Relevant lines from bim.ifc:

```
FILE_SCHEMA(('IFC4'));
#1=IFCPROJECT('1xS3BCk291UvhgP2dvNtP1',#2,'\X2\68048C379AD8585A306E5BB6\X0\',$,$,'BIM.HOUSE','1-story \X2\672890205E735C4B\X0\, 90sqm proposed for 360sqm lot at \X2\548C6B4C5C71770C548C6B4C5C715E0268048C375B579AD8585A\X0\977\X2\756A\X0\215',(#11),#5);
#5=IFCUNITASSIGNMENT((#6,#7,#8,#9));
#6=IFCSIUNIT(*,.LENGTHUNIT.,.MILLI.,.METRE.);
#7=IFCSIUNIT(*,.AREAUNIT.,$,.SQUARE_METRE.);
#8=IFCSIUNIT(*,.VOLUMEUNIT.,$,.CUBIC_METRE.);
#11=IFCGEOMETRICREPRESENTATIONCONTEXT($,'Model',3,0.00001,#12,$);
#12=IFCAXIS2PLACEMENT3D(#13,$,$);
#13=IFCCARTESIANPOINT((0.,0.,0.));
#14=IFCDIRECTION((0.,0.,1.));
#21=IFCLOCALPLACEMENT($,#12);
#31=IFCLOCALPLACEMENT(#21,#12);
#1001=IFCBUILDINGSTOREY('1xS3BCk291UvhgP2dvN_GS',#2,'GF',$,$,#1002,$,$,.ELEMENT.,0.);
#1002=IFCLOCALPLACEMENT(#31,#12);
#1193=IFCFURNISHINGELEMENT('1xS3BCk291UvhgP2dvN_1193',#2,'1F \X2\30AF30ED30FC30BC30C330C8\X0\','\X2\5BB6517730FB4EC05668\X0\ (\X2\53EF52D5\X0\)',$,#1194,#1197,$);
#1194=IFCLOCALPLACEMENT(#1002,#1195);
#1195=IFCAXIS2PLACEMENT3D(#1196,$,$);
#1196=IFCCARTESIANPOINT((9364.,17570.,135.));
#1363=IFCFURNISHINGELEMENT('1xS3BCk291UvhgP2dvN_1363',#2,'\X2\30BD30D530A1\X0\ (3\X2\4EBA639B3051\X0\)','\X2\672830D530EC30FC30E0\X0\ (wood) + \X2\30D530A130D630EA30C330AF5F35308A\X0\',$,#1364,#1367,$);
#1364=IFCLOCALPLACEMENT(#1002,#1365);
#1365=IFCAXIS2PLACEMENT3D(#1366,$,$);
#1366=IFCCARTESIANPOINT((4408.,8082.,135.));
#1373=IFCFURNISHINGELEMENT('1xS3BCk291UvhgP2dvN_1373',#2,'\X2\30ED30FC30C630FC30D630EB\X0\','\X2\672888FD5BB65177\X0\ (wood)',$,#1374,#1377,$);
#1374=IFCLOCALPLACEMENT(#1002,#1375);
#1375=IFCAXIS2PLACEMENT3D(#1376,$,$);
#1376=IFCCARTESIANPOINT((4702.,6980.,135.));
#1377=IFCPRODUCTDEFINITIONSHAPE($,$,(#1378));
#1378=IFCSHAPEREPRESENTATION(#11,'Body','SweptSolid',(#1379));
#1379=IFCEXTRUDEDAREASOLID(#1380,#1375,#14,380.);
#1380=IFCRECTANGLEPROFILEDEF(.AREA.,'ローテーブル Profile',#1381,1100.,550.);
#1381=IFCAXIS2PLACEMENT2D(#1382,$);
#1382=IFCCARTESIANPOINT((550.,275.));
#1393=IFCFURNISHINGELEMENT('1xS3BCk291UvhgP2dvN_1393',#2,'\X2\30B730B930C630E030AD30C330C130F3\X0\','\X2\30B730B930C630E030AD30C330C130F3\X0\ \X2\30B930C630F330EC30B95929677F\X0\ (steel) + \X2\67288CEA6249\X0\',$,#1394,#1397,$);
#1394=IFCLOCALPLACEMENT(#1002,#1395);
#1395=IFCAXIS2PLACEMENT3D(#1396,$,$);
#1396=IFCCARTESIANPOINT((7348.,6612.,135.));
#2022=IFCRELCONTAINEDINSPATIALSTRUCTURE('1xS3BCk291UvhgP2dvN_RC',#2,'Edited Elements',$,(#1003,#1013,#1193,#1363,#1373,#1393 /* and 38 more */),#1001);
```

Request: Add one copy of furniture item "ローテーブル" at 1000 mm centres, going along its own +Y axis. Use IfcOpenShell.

```python
import ifcopenshell
import ifcopenshell.api.geometry
import ifcopenshell.api.root
import ifcopenshell.util.element
import ifcopenshell.util.placement

model = ifcopenshell.open("bim.ifc")


def reuse_history(source, copy):
    """copy_class also copies each property set's owner history, people and application; keep the originals."""
    for rel in copy.IsDefinedBy:
        if rel.is_a("IfcRelDefinesByProperties") and (history := rel.RelatingPropertyDefinition.OwnerHistory):
            rel.RelatingPropertyDefinition.OwnerHistory = source.OwnerHistory
            ifcopenshell.util.element.remove_deep2(model, history)


source = model.by_id(1373)
base = ifcopenshell.util.placement.get_local_placement(source.ObjectPlacement)
step = base[:3, 1] * 1000.0

for i in range(1, 2):
    copy = ifcopenshell.api.root.copy_class(model, product=source)
    copy.Representation = ifcopenshell.util.element.copy_deep(
        model, source.Representation, exclude=["IfcGeometricRepresentationContext", "IfcRepresentationMap"]
    )
    reuse_history(source, copy)
    matrix = base.copy()
    matrix[:3, 3] += i * step
    print("added at", matrix[:3, 3].round(3) + 0.0)
    ifcopenshell.api.geometry.edit_object_placement(model, product=copy, matrix=matrix, is_si=False)

model.write("bim-out.ifc")
```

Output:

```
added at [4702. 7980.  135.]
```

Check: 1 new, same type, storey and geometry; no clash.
